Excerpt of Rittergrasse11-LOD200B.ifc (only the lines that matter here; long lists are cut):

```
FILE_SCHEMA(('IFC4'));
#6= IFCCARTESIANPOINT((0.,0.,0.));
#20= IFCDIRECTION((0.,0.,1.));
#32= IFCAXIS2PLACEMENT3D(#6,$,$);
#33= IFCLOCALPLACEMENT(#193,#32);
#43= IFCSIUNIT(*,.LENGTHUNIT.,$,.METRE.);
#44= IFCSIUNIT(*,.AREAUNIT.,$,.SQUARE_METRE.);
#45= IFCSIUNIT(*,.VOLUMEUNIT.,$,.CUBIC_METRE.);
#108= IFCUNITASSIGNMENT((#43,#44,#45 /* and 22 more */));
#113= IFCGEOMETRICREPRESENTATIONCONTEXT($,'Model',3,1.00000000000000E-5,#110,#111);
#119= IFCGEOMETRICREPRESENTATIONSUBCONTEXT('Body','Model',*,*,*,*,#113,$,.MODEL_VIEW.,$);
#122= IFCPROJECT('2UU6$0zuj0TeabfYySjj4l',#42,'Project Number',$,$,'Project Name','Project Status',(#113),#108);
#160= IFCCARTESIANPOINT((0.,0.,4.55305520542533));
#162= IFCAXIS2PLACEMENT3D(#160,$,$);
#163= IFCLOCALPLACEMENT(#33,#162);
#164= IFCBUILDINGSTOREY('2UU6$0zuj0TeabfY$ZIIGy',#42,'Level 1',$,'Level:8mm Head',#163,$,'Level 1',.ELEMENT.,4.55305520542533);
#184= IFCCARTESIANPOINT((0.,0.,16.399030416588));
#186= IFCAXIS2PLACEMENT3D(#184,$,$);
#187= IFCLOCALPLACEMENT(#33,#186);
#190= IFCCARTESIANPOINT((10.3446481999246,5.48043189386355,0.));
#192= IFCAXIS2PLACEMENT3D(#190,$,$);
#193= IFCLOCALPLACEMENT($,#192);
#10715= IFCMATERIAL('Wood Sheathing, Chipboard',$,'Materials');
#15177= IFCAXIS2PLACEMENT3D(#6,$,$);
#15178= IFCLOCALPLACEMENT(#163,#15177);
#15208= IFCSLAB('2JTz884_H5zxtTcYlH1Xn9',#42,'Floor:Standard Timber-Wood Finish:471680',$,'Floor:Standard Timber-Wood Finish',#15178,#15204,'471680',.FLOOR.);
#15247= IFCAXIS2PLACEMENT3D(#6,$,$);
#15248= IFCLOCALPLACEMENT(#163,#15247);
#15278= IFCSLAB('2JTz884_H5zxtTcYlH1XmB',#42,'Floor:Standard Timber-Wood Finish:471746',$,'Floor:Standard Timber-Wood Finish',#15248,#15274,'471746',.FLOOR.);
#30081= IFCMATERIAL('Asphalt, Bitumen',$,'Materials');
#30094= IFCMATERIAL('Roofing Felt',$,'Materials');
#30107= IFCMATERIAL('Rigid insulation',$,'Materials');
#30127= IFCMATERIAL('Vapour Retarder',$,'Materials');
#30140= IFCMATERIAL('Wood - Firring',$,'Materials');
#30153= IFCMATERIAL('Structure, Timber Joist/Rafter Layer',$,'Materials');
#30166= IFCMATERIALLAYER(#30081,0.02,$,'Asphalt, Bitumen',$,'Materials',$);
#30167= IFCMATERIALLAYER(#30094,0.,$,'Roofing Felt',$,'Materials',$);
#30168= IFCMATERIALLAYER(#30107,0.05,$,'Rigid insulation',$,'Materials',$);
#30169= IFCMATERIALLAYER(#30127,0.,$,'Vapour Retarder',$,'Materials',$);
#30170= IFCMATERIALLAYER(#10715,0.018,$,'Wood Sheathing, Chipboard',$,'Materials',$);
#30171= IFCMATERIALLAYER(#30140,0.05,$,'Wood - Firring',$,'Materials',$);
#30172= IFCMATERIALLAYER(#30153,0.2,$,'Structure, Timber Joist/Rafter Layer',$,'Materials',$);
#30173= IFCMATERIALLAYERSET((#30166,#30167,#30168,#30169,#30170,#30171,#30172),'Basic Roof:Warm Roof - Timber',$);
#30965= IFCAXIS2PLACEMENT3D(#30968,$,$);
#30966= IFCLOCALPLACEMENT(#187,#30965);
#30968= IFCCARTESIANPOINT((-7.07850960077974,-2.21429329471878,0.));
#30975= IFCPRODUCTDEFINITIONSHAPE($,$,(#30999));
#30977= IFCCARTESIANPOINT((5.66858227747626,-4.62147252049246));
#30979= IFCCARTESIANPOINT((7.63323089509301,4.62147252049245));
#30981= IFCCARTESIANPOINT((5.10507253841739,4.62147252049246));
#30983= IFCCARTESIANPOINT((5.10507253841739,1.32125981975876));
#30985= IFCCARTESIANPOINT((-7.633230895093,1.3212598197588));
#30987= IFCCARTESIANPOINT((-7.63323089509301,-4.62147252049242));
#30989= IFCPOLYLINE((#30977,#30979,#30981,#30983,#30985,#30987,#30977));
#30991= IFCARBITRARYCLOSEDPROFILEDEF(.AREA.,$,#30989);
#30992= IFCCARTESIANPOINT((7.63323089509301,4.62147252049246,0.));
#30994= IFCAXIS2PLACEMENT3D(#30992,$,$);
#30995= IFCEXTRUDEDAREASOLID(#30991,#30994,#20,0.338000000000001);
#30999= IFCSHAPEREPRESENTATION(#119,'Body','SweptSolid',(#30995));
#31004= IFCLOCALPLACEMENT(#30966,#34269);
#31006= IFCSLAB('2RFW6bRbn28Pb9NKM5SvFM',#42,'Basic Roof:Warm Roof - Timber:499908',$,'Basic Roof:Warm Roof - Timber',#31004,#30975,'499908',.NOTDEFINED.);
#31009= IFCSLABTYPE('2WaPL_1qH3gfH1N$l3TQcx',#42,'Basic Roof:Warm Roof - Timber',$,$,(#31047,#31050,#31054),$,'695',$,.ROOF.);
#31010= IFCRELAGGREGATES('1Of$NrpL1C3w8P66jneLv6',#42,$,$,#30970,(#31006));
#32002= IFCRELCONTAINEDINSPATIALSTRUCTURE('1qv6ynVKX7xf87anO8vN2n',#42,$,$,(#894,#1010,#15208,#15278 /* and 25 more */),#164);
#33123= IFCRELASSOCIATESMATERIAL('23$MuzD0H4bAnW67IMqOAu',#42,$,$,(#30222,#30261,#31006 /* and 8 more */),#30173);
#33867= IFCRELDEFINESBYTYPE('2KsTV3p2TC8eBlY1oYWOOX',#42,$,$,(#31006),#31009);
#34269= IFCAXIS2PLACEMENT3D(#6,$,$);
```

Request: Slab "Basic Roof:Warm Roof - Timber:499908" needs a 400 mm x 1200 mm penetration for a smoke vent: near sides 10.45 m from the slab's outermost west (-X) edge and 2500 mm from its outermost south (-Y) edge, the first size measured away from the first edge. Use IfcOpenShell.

```python
import numpy as np
import ifcopenshell
import ifcopenshell.api.feature
import ifcopenshell.api.geometry
import ifcopenshell.api.root
import ifcopenshell.geom
import ifcopenshell.util.placement
import ifcopenshell.util.representation
import ifcopenshell.util.shape
import ifcopenshell.util.unit

model = ifcopenshell.open("Rittergrasse11-LOD200B.ifc")
unit_scale = ifcopenshell.util.unit.calculate_unit_scale(model)
settings = ifcopenshell.geom.settings()


def volume(element):
    """Net volume in cubic metres, openings subtracted."""
    shape = ifcopenshell.geom.create_shape(settings, element)
    return ifcopenshell.util.shape.get_volume(shape.geometry)


slab = model.by_guid("2RFW6bRbn28Pb9NKM5SvFM")
before = volume(slab)

# Extent in the slab's own axes, in metres. The edges named are its -X and -Y sides.
slab_shape = ifcopenshell.geom.create_shape(settings, slab)
vertices = ifcopenshell.util.shape.get_vertices(slab_shape.geometry)
x_min, y_min, bottom = vertices.min(axis=0)
top = vertices[:, 2].max()

opening = ifcopenshell.api.root.create_entity(model, ifc_class="IfcOpeningElement", name="Smoke vent opening", predefined_type="OPENING")
context = ifcopenshell.util.representation.get_context(model, "Model", "Body", "MODEL_VIEW")
width, depth = 0.4, 1.2
outline = [(0.0, 0.0), (width, 0.0), (width, depth), (0.0, depth), (0.0, 0.0)]
# Overshoot both faces by 50 mm so the cut is clean.
shape = ifcopenshell.api.geometry.add_slab_representation(
    model, context=context, depth=top - bottom + 0.1, polyline=outline
)
ifcopenshell.api.geometry.assign_representation(model, product=opening, representation=shape)

matrix = ifcopenshell.util.placement.get_local_placement(slab.ObjectPlacement)
matrix[:, 3] = matrix @ np.append(np.array([x_min + 10.45, y_min + 2.5, bottom - 0.05]) / unit_scale, 1.0)
ifcopenshell.api.geometry.edit_object_placement(model, product=opening, matrix=matrix, is_si=False)
ifcopenshell.api.feature.add_feature(model, feature=opening, element=slab)

after = volume(slab)

print(f"slab volume {before:.3f} -> {after:.3f} m3")

model.write("Rittergrasse11-LOD200B_updated.ifc")
```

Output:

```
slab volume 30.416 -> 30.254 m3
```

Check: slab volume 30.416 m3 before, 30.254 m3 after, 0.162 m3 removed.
